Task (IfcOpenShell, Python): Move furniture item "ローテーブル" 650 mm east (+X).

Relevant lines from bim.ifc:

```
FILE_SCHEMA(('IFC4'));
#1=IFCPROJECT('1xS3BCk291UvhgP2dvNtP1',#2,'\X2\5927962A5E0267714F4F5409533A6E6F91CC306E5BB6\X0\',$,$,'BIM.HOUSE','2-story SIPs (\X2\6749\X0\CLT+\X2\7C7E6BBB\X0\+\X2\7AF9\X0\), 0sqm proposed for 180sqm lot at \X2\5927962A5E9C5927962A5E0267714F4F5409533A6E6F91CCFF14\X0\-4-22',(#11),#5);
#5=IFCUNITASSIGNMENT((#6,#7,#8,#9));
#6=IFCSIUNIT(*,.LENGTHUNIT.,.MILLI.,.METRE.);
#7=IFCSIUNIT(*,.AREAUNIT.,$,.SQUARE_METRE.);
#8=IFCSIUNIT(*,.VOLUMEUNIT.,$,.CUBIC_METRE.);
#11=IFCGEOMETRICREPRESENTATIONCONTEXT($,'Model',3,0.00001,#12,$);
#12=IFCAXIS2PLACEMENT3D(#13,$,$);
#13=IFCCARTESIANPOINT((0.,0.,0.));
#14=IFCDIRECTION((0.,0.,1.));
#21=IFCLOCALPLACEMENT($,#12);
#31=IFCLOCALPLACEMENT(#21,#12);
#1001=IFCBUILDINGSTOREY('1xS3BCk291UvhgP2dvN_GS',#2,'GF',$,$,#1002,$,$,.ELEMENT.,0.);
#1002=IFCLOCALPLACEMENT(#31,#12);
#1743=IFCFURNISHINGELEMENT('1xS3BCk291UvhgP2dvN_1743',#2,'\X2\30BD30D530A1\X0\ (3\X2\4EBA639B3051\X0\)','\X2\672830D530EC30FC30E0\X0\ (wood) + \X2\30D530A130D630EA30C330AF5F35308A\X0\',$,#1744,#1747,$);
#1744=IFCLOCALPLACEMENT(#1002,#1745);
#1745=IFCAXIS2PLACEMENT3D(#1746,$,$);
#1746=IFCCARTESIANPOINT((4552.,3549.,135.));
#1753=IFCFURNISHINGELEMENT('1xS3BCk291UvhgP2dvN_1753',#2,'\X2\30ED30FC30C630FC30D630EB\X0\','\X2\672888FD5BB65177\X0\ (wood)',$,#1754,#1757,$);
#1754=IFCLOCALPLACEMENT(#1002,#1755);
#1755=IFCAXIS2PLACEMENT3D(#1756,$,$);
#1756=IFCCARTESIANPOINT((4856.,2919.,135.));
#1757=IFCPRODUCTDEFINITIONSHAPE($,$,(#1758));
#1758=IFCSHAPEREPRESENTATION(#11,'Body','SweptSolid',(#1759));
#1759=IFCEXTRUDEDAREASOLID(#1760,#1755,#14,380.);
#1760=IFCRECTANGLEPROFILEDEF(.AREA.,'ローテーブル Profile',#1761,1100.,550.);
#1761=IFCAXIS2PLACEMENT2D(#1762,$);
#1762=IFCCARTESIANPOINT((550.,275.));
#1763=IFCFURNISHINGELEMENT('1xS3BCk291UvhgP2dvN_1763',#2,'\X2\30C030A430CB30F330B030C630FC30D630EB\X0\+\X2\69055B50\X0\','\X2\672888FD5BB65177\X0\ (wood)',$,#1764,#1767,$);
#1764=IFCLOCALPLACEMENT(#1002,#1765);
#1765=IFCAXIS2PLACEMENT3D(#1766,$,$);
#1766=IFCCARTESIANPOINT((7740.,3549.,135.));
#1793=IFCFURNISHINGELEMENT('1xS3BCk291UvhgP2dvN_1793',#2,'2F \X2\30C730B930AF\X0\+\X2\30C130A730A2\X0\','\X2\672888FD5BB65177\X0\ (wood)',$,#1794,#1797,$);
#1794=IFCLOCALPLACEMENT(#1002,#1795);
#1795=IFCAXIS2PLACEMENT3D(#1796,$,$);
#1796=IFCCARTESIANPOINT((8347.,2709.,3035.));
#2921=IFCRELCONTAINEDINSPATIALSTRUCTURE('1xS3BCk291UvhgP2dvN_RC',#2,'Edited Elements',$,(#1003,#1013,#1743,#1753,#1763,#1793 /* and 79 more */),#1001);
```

```python
import ifcopenshell
import ifcopenshell.api.geometry
import ifcopenshell.util.placement

model = ifcopenshell.open("bim.ifc")

item = model.by_id(1753)
matrix = ifcopenshell.util.placement.get_local_placement(item.ObjectPlacement)
matrix[0, 3] += 650.0
ifcopenshell.api.geometry.edit_object_placement(model, product=item, matrix=matrix, is_si=False)

print(ifcopenshell.util.placement.get_local_placement(item.ObjectPlacement).round(3) + 0.0)

model.write("bim_edited.ifc")
```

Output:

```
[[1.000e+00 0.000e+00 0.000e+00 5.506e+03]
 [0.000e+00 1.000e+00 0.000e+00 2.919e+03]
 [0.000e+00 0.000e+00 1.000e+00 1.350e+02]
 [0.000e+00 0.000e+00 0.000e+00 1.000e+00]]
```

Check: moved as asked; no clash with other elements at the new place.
